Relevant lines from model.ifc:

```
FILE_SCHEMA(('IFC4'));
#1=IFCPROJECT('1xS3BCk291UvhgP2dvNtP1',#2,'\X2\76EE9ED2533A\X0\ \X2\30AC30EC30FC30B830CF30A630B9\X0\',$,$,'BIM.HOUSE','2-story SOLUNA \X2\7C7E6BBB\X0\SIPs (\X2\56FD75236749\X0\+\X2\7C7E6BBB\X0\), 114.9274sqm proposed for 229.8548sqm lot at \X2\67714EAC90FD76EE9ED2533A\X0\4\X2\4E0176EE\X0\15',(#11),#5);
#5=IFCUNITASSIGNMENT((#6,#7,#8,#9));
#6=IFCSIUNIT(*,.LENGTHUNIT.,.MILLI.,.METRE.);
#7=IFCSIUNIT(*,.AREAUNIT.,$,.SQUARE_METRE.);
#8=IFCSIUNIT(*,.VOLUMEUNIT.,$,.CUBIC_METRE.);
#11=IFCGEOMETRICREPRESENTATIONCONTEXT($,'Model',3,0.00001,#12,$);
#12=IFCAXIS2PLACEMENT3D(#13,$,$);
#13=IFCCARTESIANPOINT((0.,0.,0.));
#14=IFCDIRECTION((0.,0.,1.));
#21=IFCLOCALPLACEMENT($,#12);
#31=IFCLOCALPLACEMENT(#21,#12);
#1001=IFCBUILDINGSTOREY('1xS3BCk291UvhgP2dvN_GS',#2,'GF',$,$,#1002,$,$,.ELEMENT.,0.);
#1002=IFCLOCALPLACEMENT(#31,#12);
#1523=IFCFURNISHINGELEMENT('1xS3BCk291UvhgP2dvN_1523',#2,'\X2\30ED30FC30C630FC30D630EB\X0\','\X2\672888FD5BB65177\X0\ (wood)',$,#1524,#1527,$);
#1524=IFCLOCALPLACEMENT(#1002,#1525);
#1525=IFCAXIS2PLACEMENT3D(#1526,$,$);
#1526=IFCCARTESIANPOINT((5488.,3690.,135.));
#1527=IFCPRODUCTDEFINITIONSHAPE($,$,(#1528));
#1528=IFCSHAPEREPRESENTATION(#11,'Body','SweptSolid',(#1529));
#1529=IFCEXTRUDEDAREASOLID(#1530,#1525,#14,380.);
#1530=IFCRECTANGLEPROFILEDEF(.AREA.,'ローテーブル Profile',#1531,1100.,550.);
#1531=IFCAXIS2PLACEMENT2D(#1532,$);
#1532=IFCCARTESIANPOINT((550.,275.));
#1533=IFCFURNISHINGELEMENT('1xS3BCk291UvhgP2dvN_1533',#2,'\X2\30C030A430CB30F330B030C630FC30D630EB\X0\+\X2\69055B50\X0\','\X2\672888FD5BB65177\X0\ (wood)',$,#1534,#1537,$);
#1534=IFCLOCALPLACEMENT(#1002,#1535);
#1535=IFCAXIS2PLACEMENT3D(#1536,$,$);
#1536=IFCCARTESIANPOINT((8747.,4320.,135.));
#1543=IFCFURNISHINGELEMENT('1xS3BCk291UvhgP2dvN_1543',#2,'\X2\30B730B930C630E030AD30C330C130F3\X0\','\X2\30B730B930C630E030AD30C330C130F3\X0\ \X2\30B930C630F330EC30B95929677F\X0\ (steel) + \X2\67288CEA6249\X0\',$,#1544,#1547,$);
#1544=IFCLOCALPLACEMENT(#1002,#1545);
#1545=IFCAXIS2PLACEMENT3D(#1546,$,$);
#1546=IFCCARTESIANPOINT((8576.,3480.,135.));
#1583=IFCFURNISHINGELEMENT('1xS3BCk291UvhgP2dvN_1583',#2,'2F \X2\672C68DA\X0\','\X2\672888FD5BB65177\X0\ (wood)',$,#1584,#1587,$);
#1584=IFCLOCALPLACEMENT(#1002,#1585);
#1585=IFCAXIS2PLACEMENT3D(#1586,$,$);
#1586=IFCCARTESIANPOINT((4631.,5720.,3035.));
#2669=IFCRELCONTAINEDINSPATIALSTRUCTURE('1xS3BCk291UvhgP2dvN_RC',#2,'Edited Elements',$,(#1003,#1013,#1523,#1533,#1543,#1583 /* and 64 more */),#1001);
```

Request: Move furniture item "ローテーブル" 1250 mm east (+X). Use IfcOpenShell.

```python
import ifcopenshell
import ifcopenshell.api.geometry
import ifcopenshell.util.placement
import ifcopenshell.util.unit

model = ifcopenshell.open("model.ifc")
unit_scale = ifcopenshell.util.unit.calculate_unit_scale(model)

item = model.by_id(1523)
matrix = ifcopenshell.util.placement.get_local_placement(item.ObjectPlacement)
matrix[0, 3] += 1.25 / unit_scale
ifcopenshell.api.geometry.edit_object_placement(model, product=item, matrix=matrix, is_si=False)

print(ifcopenshell.util.placement.get_local_placement(item.ObjectPlacement).round(3) + 0.0)

model.write("model-out.ifc")
```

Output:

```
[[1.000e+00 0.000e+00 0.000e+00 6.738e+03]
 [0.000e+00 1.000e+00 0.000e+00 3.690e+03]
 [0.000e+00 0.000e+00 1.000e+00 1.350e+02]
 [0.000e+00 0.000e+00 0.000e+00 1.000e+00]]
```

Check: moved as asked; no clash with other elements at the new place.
